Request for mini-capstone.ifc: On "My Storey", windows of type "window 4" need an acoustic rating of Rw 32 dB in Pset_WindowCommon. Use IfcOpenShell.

First a look at what the model holds.

```python
import ifcopenshell
import ifcopenshell.util.element

model = ifcopenshell.open("mini-capstone.ifc")
print(model.schema)
storey = next(s for s in model.by_type("IfcBuildingStorey") if s.Name == "My Storey")
windows = [e for e in ifcopenshell.util.element.get_decomposition(storey) if e.is_a("IfcWindow")]
seen = {}
for e in windows:
    element_type = ifcopenshell.util.element.get_type(e)
    key = (element_type.Name if element_type != e and element_type else None, ifcopenshell.util.element.get_pset(e, "Pset_WindowCommon", "AcousticRating"))
    seen[key] = seen.get(key, 0) + 1
for (name, value), count in sorted(seen.items(), key=str):
    print(count, "x", name, "|", value)
```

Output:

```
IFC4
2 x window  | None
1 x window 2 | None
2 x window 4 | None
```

```python
import ifcopenshell
import ifcopenshell.api.pset
import ifcopenshell.util.element

model = ifcopenshell.open("mini-capstone.ifc")

storey = next(s for s in model.by_type("IfcBuildingStorey") if s.Name == "My Storey")
windows = [e for e in ifcopenshell.util.element.get_decomposition(storey) if e.is_a("IfcWindow")]

count = 0
for e in windows:
    element_type = ifcopenshell.util.element.get_type(e)
    if element_type in (None, e) or element_type.Name != "window 4":
        continue
    # add_pset returns the element's existing set when there is one.
    pset = ifcopenshell.api.pset.add_pset(model, product=e, name="Pset_WindowCommon")
    ifcopenshell.api.pset.edit_pset(model, pset=pset, properties={"AcousticRating": "Rw 32 dB"})
    count += 1

print(count, "windows updated")

model.write("mini-capstone_updated.ifc")
```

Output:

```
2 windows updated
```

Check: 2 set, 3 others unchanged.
